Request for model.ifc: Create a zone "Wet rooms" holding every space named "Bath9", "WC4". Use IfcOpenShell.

First a look at what the model holds.

```python
import ifcopenshell

model = ifcopenshell.open("model.ifc")
print(model.schema)
seen = {}
for space in model.by_type("IfcSpace"):
    seen[space.Name] = seen.get(space.Name, 0) + 1
for name, count in sorted(seen.items(), key=str):
    print(count, "x", name)
print("zones:", [z.Name for z in model.by_type("IfcZone")][:20])
```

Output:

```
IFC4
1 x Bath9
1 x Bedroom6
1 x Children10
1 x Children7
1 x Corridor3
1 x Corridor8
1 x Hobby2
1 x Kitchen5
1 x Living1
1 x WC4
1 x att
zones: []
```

```python
import ifcopenshell
import ifcopenshell.api.group
import ifcopenshell.api.root

model = ifcopenshell.open("model.ifc")

names = {"Bath9", "WC4"}
spaces = [s for s in model.by_type("IfcSpace") if s.Name in names]

zone = ifcopenshell.api.root.create_entity(model, ifc_class="IfcZone", name="Wet rooms")
ifcopenshell.api.group.assign_group(model, products=spaces, group=zone)
print(len(spaces), "spaces in", zone.Name)

model.write("model_v2.ifc")
```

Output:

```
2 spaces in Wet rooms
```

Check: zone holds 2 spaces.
